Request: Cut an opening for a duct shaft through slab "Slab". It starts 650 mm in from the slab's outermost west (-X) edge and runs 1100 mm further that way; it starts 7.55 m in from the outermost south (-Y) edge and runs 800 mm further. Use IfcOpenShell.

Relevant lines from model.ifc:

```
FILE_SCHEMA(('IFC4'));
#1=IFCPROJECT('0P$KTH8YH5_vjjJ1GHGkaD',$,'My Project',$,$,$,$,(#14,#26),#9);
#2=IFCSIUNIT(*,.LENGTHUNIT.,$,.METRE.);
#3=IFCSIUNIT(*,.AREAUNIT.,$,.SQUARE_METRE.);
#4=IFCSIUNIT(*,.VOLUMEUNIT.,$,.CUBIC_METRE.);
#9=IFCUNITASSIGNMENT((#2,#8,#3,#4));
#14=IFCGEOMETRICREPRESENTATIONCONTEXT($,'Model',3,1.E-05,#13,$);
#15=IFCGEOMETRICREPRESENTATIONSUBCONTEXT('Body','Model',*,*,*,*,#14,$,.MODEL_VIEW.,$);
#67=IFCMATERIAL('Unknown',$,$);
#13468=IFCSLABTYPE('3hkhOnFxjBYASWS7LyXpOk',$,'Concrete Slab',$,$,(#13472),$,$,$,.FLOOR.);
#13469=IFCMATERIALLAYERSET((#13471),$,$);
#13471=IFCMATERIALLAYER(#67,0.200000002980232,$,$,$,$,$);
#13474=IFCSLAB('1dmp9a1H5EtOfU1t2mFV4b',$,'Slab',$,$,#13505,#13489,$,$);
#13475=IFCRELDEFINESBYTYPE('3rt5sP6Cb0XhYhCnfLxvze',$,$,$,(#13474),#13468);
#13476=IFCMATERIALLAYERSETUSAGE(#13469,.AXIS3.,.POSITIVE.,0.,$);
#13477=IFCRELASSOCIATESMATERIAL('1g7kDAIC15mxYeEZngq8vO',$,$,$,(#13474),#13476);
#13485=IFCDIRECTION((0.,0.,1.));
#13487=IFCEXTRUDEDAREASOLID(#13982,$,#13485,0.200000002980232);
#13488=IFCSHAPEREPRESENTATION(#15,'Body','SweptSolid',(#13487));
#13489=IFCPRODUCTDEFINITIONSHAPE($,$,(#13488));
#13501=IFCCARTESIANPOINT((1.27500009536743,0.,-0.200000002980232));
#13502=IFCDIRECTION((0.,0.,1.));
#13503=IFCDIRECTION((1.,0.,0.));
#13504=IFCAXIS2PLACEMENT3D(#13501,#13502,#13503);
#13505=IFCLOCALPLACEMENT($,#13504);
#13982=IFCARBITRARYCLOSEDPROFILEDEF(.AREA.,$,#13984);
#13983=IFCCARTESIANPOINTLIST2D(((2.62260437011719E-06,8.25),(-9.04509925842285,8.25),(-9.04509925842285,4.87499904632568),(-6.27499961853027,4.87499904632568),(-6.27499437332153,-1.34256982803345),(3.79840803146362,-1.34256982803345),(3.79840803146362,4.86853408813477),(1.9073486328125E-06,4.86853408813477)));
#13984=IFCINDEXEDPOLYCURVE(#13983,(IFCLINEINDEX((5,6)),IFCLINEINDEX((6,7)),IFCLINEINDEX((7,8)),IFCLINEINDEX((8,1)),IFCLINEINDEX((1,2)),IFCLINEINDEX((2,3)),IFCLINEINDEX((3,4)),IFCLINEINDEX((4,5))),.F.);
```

```python
import numpy as np
import ifcopenshell
import ifcopenshell.api.feature
import ifcopenshell.api.geometry
import ifcopenshell.api.root
import ifcopenshell.geom
import ifcopenshell.util.placement
import ifcopenshell.util.representation
import ifcopenshell.util.shape
import ifcopenshell.util.unit

model = ifcopenshell.open("model.ifc")
unit_scale = ifcopenshell.util.unit.calculate_unit_scale(model)
settings = ifcopenshell.geom.settings()


def volume(element):
    """Net volume in cubic metres, openings subtracted."""
    shape = ifcopenshell.geom.create_shape(settings, element)
    return ifcopenshell.util.shape.get_volume(shape.geometry)


slab = model.by_guid("1dmp9a1H5EtOfU1t2mFV4b")
before = volume(slab)

# Extent in the slab's own axes, in metres. The edges named are its -X and -Y sides.
slab_shape = ifcopenshell.geom.create_shape(settings, slab)
vertices = ifcopenshell.util.shape.get_vertices(slab_shape.geometry)
x_min, y_min, bottom = vertices.min(axis=0)
top = vertices[:, 2].max()

opening = ifcopenshell.api.root.create_entity(model, ifc_class="IfcOpeningElement", name="Duct shaft opening", predefined_type="OPENING")
context = ifcopenshell.util.representation.get_context(model, "Model", "Body", "MODEL_VIEW")
width, depth = 1.1, 0.8
outline = [(0.0, 0.0), (width, 0.0), (width, depth), (0.0, depth), (0.0, 0.0)]
# Overshoot both faces by 50 mm so the cut is clean.
shape = ifcopenshell.api.geometry.add_slab_representation(
    model, context=context, depth=top - bottom + 0.1, polyline=outline
)
ifcopenshell.api.geometry.assign_representation(model, product=opening, representation=shape)

matrix = ifcopenshell.util.placement.get_local_placement(slab.ObjectPlacement)
matrix[:, 3] = matrix @ np.append(np.array([x_min + 0.65, y_min + 7.55, bottom - 0.05]) / unit_scale, 1.0)
ifcopenshell.api.geometry.edit_object_placement(model, product=opening, matrix=matrix, is_si=False)
ifcopenshell.api.feature.add_feature(model, feature=opening, element=slab)

after = volume(slab)

print(f"slab volume {before:.3f} -> {after:.3f} m3")

model.write("model-out.ifc")
```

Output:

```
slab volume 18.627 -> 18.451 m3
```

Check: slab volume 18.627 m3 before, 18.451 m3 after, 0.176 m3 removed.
